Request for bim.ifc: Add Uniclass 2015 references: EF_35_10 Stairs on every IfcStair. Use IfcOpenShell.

First a look at what the model holds.

```python
import ifcopenshell

model = ifcopenshell.open("bim.ifc")
print(model.schema)
print("classifications:", [c.Name for c in model.by_type("IfcClassification")])
for ifc_class in ("IfcDoor", "IfcRoof", "IfcStair", "IfcWall", "IfcWindow"):
    print(ifc_class, len(model.by_type(ifc_class)))
```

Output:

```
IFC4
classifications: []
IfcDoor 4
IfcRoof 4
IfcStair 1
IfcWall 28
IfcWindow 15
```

```python
import ifcopenshell
import ifcopenshell.api.classification

model = ifcopenshell.open("bim.ifc")

system = ifcopenshell.api.classification.add_classification(model, classification="Uniclass 2015")

codes = {
    "IfcStair": ("EF_35_10", "Stairs"),
}
for ifc_class, (code, name) in codes.items():
    products = model.by_type(ifc_class)
    ifcopenshell.api.classification.add_reference(
        model, products=products, classification=system, identification=code, name=name
    )
    print(code, len(products))

model.write("bim-out.ifc")
```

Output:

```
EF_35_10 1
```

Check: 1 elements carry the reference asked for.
